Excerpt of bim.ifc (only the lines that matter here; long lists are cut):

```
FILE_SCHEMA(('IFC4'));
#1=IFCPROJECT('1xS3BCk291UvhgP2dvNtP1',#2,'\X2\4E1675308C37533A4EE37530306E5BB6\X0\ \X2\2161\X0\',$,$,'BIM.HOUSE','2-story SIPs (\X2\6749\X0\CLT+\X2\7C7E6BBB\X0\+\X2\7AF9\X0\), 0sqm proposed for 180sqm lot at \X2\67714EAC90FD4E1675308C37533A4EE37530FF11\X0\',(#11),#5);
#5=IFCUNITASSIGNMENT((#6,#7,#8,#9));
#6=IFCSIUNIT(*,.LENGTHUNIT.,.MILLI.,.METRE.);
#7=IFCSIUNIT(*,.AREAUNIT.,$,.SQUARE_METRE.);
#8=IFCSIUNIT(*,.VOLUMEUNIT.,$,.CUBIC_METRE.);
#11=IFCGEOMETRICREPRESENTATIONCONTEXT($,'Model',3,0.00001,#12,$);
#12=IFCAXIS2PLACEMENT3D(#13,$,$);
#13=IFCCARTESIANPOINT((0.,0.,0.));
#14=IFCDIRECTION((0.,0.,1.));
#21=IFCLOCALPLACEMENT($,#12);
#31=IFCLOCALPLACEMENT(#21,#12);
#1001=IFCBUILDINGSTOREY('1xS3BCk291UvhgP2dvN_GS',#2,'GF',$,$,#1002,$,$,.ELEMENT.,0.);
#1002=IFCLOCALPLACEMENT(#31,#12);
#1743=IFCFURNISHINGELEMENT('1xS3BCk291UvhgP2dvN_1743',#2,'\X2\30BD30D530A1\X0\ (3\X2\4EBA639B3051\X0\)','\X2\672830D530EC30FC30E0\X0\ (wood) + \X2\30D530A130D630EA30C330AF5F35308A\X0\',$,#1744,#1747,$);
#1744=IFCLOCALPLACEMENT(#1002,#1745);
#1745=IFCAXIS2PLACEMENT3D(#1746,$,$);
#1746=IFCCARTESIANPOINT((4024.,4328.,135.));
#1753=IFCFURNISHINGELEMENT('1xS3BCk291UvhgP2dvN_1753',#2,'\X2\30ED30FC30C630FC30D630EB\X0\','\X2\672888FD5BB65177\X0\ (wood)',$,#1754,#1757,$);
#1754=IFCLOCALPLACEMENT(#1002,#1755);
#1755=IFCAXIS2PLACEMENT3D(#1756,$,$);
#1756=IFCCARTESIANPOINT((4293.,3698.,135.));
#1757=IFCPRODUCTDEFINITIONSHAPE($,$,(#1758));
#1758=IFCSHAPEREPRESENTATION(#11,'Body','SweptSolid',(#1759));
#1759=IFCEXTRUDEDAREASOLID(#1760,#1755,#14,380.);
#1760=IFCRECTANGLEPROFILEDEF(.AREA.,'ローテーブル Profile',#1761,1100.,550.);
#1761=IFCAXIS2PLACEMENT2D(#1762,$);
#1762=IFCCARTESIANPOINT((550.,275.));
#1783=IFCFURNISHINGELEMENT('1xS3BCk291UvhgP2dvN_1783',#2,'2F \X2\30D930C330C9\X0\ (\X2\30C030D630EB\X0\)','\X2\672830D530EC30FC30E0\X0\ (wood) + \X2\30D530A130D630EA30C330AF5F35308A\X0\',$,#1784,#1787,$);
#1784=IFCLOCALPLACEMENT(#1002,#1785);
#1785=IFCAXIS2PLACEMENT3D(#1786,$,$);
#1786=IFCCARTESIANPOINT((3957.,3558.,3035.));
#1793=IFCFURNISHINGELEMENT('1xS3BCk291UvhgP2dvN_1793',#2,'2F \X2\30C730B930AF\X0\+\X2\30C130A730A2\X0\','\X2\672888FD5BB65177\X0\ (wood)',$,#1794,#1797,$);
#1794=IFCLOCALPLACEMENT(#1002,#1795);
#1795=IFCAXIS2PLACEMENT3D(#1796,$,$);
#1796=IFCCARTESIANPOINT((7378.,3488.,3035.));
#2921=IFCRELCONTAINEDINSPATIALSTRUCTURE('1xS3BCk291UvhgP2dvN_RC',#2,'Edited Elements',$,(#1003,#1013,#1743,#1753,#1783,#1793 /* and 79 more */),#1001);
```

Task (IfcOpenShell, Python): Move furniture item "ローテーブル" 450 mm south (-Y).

```python
import ifcopenshell
import ifcopenshell.api.geometry
import ifcopenshell.util.placement
import ifcopenshell.util.unit

model = ifcopenshell.open("bim.ifc")
unit_scale = ifcopenshell.util.unit.calculate_unit_scale(model)

item = model.by_guid("1xS3BCk291UvhgP2dvN_1753")
matrix = ifcopenshell.util.placement.get_local_placement(item.ObjectPlacement)
matrix[1, 3] -= 0.45 / unit_scale
ifcopenshell.api.geometry.edit_object_placement(model, product=item, matrix=matrix, is_si=False)

print(ifcopenshell.util.placement.get_local_placement(item.ObjectPlacement).round(3) + 0.0)

model.write("bim_rev.ifc")
```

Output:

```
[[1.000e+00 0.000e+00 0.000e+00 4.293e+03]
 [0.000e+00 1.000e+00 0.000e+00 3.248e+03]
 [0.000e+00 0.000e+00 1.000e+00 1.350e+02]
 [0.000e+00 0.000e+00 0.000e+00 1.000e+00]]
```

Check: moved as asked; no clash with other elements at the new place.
